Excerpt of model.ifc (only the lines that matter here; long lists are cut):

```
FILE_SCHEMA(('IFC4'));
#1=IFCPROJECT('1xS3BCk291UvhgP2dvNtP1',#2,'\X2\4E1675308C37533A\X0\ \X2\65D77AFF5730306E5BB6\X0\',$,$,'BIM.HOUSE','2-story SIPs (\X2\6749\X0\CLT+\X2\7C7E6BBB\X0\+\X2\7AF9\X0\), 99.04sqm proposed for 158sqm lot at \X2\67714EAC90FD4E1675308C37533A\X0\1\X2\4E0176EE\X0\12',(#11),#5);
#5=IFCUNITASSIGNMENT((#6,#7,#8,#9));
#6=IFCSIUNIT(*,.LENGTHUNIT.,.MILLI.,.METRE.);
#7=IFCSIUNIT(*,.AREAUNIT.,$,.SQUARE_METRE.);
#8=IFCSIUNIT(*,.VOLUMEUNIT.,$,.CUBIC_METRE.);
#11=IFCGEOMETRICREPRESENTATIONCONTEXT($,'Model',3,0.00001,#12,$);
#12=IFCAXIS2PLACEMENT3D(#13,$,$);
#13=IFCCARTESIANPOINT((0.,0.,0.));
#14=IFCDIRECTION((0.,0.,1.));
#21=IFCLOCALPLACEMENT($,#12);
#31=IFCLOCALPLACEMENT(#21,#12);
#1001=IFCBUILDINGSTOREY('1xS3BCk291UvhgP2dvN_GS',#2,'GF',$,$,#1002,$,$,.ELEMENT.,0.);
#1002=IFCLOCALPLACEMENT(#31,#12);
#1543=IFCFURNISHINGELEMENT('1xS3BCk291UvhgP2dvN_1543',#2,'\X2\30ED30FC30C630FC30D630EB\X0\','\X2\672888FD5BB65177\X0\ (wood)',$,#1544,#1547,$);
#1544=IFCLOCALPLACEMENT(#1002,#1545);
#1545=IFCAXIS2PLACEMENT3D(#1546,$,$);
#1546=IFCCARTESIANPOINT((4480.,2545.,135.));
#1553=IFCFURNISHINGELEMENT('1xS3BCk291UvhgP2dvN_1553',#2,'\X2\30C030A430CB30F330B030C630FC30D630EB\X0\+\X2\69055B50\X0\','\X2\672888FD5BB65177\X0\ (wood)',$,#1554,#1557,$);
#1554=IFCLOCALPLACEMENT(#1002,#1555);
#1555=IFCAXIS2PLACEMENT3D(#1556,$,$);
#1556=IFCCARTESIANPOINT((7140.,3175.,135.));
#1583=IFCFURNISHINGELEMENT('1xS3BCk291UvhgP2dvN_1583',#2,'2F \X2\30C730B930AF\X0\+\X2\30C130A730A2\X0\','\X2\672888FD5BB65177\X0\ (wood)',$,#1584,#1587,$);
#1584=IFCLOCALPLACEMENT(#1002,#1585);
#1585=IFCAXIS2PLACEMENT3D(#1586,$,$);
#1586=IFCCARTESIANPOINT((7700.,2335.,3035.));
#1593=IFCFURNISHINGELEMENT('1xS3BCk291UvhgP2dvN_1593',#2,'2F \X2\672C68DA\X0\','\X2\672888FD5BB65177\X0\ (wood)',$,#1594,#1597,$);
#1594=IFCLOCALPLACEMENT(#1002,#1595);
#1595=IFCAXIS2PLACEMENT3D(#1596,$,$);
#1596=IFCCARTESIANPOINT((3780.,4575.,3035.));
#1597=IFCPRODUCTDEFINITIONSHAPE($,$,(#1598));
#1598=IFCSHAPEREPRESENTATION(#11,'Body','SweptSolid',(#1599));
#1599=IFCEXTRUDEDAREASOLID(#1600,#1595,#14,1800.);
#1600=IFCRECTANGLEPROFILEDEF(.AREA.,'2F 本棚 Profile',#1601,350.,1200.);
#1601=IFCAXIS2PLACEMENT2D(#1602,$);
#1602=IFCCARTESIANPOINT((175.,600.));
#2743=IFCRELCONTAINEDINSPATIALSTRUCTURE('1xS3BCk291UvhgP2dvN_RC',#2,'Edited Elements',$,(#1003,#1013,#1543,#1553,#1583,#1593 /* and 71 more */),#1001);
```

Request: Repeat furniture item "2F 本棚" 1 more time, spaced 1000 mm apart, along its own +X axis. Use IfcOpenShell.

```python
import ifcopenshell
import ifcopenshell.api.geometry
import ifcopenshell.api.root
import ifcopenshell.util.element
import ifcopenshell.util.placement
import ifcopenshell.util.unit

model = ifcopenshell.open("model.ifc")
unit_scale = ifcopenshell.util.unit.calculate_unit_scale(model)


def reuse_history(source, copy):
    """copy_class also copies each property set's owner history, people and application; keep the originals."""
    for rel in copy.IsDefinedBy:
        if rel.is_a("IfcRelDefinesByProperties") and (history := rel.RelatingPropertyDefinition.OwnerHistory):
            rel.RelatingPropertyDefinition.OwnerHistory = source.OwnerHistory
            ifcopenshell.util.element.remove_deep2(model, history)


source = model.by_id(1593)
base = ifcopenshell.util.placement.get_local_placement(source.ObjectPlacement)
step = base[:3, 0] * 1 / unit_scale

for i in range(1, 2):
    copy = ifcopenshell.api.root.copy_class(model, product=source)
    copy.Representation = ifcopenshell.util.element.copy_deep(
        model, source.Representation, exclude=["IfcGeometricRepresentationContext", "IfcRepresentationMap"]
    )
    reuse_history(source, copy)
    matrix = base.copy()
    matrix[:3, 3] += i * step
    print("added at", matrix[:3, 3].round(3) + 0.0)
    ifcopenshell.api.geometry.edit_object_placement(model, product=copy, matrix=matrix, is_si=False)

model.write("model-out.ifc")
```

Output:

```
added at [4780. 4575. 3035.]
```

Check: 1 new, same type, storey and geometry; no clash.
